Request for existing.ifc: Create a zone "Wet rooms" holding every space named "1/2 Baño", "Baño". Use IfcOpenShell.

First a look at what the model holds.

```python
import ifcopenshell

model = ifcopenshell.open("existing.ifc")
print(model.schema)
seen = {}
for space in model.by_type("IfcSpace"):
    seen[space.LongName] = seen.get(space.LongName, 0) + 1
for name, count in sorted(seen.items(), key=str):
    print(count, "x", name)
print("zones:", [z.Name for z in model.by_type("IfcZone")][:20])
```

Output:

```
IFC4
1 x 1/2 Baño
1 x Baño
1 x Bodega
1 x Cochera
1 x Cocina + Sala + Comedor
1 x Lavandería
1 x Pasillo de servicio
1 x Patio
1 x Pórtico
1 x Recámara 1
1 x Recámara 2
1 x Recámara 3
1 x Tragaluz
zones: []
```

```python
import ifcopenshell
import ifcopenshell.api.group
import ifcopenshell.api.root

model = ifcopenshell.open("existing.ifc")

names = {"1/2 Baño", "Baño"}
spaces = [s for s in model.by_type("IfcSpace") if s.LongName in names]

zone = ifcopenshell.api.root.create_entity(model, ifc_class="IfcZone", name="Wet rooms")
ifcopenshell.api.group.assign_group(model, products=spaces, group=zone)
print(len(spaces), "spaces in", zone.Name)

model.write("existing_rev.ifc")
```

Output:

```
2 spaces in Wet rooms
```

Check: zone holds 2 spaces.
